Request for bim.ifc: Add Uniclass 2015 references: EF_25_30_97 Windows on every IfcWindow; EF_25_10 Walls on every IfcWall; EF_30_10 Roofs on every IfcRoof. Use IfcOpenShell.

First a look at what the model holds.

```python
import ifcopenshell

model = ifcopenshell.open("bim.ifc")
print(model.schema)
print("classifications:", [c.Name for c in model.by_type("IfcClassification")])
for ifc_class in ("IfcDoor", "IfcRoof", "IfcStair", "IfcWall", "IfcWindow"):
    print(ifc_class, len(model.by_type(ifc_class)))
```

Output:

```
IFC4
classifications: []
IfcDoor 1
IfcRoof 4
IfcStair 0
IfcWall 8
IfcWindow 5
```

```python
import ifcopenshell
import ifcopenshell.api.classification

model = ifcopenshell.open("bim.ifc")

system = ifcopenshell.api.classification.add_classification(model, classification="Uniclass 2015")

codes = {
    "IfcWindow": ("EF_25_30_97", "Windows"),
    "IfcWall": ("EF_25_10", "Walls"),
    "IfcRoof": ("EF_30_10", "Roofs"),
}
for ifc_class, (code, name) in codes.items():
    products = model.by_type(ifc_class)
    ifcopenshell.api.classification.add_reference(
        model, products=products, classification=system, identification=code, name=name
    )
    print(code, len(products))

model.write("bim_v2.ifc")
```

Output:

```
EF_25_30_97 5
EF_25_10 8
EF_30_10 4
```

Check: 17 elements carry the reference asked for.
